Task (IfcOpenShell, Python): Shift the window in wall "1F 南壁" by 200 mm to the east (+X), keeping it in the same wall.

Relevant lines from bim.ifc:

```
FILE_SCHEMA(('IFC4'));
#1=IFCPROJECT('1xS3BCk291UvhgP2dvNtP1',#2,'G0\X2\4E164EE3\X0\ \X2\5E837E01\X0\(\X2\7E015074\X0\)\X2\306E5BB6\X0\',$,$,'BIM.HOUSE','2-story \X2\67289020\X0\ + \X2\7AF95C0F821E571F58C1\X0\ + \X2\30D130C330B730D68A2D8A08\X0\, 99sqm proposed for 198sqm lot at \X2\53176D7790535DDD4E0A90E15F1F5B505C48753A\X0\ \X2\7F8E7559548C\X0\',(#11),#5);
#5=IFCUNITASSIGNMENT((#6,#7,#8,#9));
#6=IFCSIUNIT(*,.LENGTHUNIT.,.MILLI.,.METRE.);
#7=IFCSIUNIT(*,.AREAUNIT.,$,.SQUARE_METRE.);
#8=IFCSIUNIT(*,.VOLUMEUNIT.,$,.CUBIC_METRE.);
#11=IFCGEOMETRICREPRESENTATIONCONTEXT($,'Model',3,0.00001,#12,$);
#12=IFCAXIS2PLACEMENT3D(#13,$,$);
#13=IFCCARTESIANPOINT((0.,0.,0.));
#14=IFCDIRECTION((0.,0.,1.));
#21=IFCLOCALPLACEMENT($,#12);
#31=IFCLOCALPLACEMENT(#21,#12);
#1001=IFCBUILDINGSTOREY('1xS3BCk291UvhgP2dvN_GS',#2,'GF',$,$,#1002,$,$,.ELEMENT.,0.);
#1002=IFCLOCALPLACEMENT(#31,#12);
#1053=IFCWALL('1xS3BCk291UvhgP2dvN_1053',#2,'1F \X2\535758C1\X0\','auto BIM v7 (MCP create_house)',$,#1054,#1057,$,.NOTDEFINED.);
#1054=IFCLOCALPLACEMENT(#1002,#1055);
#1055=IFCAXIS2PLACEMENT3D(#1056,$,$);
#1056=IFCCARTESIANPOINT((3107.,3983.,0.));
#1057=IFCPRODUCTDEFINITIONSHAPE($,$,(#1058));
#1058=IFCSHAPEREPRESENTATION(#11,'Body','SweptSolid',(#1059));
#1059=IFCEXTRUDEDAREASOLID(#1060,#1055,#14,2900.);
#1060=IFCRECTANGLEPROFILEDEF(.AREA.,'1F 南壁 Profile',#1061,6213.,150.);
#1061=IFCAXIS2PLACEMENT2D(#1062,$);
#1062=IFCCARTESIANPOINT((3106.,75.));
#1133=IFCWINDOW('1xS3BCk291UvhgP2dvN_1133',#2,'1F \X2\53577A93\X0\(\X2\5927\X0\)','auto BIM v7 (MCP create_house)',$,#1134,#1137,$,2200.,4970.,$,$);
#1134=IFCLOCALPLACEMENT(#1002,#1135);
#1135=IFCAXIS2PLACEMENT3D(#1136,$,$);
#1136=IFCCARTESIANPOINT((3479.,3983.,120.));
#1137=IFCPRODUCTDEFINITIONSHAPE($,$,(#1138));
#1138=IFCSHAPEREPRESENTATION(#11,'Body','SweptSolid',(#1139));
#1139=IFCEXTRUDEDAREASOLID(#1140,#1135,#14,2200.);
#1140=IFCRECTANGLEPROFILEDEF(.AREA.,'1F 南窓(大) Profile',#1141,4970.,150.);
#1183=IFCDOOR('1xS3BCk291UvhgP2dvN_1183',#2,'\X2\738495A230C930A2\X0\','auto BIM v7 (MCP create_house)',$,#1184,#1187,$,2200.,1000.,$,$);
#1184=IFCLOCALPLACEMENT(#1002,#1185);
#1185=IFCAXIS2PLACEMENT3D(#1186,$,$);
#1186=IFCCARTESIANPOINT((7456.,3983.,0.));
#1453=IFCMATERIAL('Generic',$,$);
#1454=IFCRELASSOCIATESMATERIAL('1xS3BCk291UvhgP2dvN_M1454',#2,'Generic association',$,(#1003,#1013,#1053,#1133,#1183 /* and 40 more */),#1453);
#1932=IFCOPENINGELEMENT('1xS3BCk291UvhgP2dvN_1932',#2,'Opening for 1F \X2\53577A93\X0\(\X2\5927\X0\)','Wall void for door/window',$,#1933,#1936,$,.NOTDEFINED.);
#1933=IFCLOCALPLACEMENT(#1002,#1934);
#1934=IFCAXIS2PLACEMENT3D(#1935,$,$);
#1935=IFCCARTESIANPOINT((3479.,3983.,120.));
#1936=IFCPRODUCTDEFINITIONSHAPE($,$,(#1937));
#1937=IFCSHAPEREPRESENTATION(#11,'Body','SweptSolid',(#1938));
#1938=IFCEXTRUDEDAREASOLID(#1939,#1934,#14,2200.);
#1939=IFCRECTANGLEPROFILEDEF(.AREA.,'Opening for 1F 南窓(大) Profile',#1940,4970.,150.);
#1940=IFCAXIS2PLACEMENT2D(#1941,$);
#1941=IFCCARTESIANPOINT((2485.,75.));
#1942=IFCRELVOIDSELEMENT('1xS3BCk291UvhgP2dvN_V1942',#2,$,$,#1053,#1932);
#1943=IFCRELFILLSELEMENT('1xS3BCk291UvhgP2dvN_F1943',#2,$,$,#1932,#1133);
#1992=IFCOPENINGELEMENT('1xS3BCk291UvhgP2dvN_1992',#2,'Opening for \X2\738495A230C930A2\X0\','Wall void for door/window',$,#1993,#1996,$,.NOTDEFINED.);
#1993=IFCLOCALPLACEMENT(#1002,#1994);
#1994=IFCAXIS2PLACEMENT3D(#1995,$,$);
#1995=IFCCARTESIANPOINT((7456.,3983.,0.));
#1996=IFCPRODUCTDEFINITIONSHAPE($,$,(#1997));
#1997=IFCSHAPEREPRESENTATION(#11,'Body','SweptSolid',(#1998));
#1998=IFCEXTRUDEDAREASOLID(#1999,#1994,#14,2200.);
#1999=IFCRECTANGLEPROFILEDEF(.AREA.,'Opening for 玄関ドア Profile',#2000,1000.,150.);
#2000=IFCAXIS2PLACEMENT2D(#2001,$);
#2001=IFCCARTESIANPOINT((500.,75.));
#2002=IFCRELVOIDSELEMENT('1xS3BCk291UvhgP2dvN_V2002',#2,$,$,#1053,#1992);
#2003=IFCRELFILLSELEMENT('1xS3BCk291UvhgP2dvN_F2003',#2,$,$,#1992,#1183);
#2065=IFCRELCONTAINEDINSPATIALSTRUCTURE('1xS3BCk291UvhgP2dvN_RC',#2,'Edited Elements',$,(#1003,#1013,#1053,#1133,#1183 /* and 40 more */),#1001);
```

```python
import ifcopenshell
import ifcopenshell.api.geometry
import ifcopenshell.util.placement

model = ifcopenshell.open("bim.ifc")

window = model.by_guid("1xS3BCk291UvhgP2dvN_1133")
opening = window.FillsVoids[0].RelatingOpeningElement
wall = opening.VoidsElements[0].RelatingBuildingElement

wall_matrix = ifcopenshell.util.placement.get_local_placement(wall.ObjectPlacement)
shift = wall_matrix[:3, 0] * 200.0
before = ifcopenshell.util.placement.get_local_placement(window.ObjectPlacement)[:3, 3].copy()

# The window is not placed relative to its opening, so move both.
for product in (opening, window):
    matrix = ifcopenshell.util.placement.get_local_placement(product.ObjectPlacement)
    matrix[:3, 3] += shift
    ifcopenshell.api.geometry.edit_object_placement(model, product=product, matrix=matrix, is_si=False)

after = ifcopenshell.util.placement.get_local_placement(window.ObjectPlacement)[:3, 3]
print("window moved by", (after - before).round(3) + 0.0)

model.write("bim_edited.ifc")
```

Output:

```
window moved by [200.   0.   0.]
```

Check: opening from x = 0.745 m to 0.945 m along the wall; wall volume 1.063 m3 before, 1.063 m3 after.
